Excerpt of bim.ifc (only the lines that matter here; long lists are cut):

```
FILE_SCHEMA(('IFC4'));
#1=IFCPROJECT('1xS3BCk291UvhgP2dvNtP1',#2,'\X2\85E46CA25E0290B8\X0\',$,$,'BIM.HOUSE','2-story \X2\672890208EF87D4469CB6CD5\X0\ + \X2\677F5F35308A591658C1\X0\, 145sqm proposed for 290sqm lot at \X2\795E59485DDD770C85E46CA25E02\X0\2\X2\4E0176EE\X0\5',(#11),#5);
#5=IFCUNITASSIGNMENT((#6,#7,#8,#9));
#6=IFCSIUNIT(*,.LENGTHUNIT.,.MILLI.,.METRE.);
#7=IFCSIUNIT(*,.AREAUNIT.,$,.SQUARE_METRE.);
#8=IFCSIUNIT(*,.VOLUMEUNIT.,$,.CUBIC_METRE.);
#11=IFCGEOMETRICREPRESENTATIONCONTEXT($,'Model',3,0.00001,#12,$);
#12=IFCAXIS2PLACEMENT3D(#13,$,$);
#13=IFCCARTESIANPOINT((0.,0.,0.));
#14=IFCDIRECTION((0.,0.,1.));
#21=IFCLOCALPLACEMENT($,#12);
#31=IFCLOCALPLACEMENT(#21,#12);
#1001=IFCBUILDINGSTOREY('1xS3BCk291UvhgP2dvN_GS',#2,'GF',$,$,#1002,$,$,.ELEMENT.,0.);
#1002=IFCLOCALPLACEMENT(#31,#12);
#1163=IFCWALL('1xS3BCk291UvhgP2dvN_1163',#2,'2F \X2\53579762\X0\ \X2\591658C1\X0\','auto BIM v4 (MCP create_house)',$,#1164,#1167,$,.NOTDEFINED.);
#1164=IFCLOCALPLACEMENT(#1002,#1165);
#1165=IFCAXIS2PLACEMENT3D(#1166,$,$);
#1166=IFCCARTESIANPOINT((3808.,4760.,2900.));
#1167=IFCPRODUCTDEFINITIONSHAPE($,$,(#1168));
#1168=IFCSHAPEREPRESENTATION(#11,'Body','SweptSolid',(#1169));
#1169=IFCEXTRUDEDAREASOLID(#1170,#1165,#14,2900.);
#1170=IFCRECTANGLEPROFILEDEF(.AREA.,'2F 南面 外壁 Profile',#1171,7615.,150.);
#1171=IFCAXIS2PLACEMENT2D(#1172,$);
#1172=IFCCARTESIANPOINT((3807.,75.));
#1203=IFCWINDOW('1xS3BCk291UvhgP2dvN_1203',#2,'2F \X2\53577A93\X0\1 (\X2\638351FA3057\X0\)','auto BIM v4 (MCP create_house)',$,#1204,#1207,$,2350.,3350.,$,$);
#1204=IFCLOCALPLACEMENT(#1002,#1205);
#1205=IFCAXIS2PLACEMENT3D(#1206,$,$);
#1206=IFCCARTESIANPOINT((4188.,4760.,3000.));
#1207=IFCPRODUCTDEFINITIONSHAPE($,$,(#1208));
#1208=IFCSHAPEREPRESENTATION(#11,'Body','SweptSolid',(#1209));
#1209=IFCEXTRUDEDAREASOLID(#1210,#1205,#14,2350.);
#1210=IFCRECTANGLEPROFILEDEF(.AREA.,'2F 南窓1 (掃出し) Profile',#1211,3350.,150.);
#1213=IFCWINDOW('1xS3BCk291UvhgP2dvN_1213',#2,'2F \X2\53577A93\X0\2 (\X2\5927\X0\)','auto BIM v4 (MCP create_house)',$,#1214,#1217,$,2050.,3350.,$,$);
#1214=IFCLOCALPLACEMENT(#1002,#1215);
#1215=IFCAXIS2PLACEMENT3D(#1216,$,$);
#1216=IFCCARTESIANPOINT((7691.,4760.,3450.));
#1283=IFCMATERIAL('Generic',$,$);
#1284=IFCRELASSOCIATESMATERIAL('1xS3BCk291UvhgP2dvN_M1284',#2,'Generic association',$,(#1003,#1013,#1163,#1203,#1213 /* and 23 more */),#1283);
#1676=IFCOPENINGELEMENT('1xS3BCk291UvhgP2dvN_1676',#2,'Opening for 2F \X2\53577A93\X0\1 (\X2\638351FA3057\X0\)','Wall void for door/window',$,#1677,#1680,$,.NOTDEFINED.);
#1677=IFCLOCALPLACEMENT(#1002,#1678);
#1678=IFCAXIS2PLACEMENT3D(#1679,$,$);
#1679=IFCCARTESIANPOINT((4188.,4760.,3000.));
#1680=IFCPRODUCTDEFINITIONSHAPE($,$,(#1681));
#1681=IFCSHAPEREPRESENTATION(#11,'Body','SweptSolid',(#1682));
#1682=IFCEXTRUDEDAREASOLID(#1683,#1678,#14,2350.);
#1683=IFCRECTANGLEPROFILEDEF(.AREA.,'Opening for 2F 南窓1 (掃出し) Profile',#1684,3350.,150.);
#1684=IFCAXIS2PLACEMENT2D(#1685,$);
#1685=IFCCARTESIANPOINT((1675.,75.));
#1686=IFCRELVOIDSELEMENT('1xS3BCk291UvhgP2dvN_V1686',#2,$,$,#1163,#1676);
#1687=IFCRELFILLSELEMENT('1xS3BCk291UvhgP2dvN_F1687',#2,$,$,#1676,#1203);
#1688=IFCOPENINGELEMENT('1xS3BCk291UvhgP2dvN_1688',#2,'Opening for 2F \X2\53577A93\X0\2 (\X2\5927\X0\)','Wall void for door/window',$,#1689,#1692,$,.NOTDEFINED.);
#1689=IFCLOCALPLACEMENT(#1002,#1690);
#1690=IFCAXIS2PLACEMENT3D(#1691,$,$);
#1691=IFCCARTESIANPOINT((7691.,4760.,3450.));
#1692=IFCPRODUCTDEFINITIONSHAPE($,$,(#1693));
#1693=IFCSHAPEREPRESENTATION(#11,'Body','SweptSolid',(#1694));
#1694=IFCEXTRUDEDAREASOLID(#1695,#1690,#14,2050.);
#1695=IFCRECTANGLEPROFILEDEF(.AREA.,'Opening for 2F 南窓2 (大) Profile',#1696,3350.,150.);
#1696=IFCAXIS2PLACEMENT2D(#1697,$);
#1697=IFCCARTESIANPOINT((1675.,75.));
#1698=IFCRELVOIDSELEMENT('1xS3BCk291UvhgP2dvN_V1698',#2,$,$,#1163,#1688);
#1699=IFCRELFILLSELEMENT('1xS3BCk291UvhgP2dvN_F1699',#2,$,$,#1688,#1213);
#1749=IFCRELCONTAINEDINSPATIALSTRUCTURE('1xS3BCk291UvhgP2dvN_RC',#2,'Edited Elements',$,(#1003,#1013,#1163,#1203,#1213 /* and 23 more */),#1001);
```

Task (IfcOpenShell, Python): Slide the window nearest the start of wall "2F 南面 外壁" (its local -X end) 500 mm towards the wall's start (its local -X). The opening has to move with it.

```python
import ifcopenshell
import ifcopenshell.api.geometry
import ifcopenshell.util.placement

model = ifcopenshell.open("bim.ifc")

window = model.by_guid("1xS3BCk291UvhgP2dvN_1203")
opening = window.FillsVoids[0].RelatingOpeningElement
wall = opening.VoidsElements[0].RelatingBuildingElement

wall_matrix = ifcopenshell.util.placement.get_local_placement(wall.ObjectPlacement)
shift = wall_matrix[:3, 0] * -500.0
before = ifcopenshell.util.placement.get_local_placement(window.ObjectPlacement)[:3, 3].copy()

# The window is not placed relative to its opening, so move both.
for product in (opening, window):
    matrix = ifcopenshell.util.placement.get_local_placement(product.ObjectPlacement)
    matrix[:3, 3] += shift
    ifcopenshell.api.geometry.edit_object_placement(model, product=product, matrix=matrix, is_si=False)

after = ifcopenshell.util.placement.get_local_placement(window.ObjectPlacement)[:3, 3]
print("window moved by", (after - before).round(3) + 0.0)

model.write("bim_updated.ifc")
```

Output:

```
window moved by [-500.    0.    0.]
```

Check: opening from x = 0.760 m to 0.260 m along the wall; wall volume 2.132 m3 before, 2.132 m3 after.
